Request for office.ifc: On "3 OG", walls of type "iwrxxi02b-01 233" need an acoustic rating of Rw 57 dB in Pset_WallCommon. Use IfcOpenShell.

First a look at what the model holds.

```python
import ifcopenshell
import ifcopenshell.util.element

model = ifcopenshell.open("office.ifc")
print(model.schema)
storey = next(s for s in model.by_type("IfcBuildingStorey") if s.Name == "3 OG")
walls = [e for e in ifcopenshell.util.element.get_decomposition(storey) if e.is_a("IfcWall")]
seen = {}
for e in walls:
    element_type = ifcopenshell.util.element.get_type(e)
    key = (element_type.Name if element_type != e and element_type else None, ifcopenshell.util.element.get_pset(e, "Pset_WallCommon", "AcousticRating"))
    seen[key] = seen.get(key, 0) + 1
for (name, value), count in sorted(seen.items(), key=str):
    print(count, "x", name, "|", value)
```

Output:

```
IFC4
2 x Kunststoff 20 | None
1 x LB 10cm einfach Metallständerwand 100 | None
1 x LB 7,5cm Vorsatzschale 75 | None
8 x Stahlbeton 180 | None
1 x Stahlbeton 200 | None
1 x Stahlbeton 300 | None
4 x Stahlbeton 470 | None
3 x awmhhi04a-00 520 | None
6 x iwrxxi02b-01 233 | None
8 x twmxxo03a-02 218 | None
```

```python
import ifcopenshell
import ifcopenshell.api.pset
import ifcopenshell.util.element

model = ifcopenshell.open("office.ifc")

storey = next(s for s in model.by_type("IfcBuildingStorey") if s.Name == "3 OG")
walls = [e for e in ifcopenshell.util.element.get_decomposition(storey) if e.is_a("IfcWall")]

count = 0
for e in walls:
    element_type = ifcopenshell.util.element.get_type(e)
    if element_type in (None, e) or element_type.Name != "iwrxxi02b-01 233":
        continue
    # add_pset returns the element's existing set when there is one.
    pset = ifcopenshell.api.pset.add_pset(model, product=e, name="Pset_WallCommon")
    ifcopenshell.api.pset.edit_pset(model, pset=pset, properties={"AcousticRating": "Rw 57 dB"})
    count += 1

print(count, "walls updated")

model.write("office_rev.ifc")
```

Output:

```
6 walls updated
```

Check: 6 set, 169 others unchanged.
